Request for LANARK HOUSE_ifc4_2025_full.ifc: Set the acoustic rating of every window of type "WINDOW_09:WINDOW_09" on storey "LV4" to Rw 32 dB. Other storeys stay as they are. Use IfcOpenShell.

First a look at what the model holds.

```python
import ifcopenshell
import ifcopenshell.util.element

model = ifcopenshell.open("LANARK HOUSE_ifc4_2025_full.ifc")
print(model.schema)
storey = next(s for s in model.by_type("IfcBuildingStorey") if s.Name == "LV4")
windows = [e for e in ifcopenshell.util.element.get_decomposition(storey) if e.is_a("IfcWindow")]
seen = {}
for e in windows:
    element_type = ifcopenshell.util.element.get_type(e)
    key = (element_type.Name if element_type != e and element_type else None, ifcopenshell.util.element.get_pset(e, "Pset_WindowCommon", "AcousticRating"))
    seen[key] = seen.get(key, 0) + 1
for (name, value), count in sorted(seen.items(), key=str):
    print(count, "x", name, "|", value)
```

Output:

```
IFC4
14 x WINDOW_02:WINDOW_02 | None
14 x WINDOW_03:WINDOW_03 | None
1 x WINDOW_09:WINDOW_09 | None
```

```python
import ifcopenshell
import ifcopenshell.api.pset
import ifcopenshell.util.element

model = ifcopenshell.open("LANARK HOUSE_ifc4_2025_full.ifc")

storey = next(s for s in model.by_type("IfcBuildingStorey") if s.Name == "LV4")
windows = [e for e in ifcopenshell.util.element.get_decomposition(storey) if e.is_a("IfcWindow")]

count = 0
for e in windows:
    element_type = ifcopenshell.util.element.get_type(e)
    if element_type in (None, e) or element_type.Name != "WINDOW_09:WINDOW_09":
        continue
    # add_pset returns the element's existing set when there is one.
    pset = ifcopenshell.api.pset.add_pset(model, product=e, name="Pset_WindowCommon")
    ifcopenshell.api.pset.edit_pset(model, pset=pset, properties={"AcousticRating": "Rw 32 dB"})
    count += 1

print(count, "windows updated")

model.write("LANARK HOUSE_ifc4_2025_full-out.ifc")
```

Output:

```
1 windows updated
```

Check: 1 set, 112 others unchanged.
